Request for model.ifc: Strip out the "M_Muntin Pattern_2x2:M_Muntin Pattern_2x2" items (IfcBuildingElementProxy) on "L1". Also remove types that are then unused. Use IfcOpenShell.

First a look at what the model holds.

```python
import ifcopenshell
import ifcopenshell.util.element

model = ifcopenshell.open("model.ifc")
print(model.schema)
storey = next(s for s in model.by_type("IfcBuildingStorey") if s.Name == "L1")
proxies = [e for e in ifcopenshell.util.element.get_decomposition(storey) if e.is_a("IfcBuildingElementProxy")]
seen = {}
for e in proxies:
    element_type = ifcopenshell.util.element.get_type(e)
    name = element_type.Name if element_type not in (None, e) else None
    seen[name] = seen.get(name, 0) + 1
for name, count in sorted(seen.items(), key=str):
    print(count, "x", name)
```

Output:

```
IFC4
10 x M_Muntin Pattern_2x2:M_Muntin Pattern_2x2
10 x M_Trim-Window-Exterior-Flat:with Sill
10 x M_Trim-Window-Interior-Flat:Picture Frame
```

```python
import ifcopenshell
import ifcopenshell.api.root
import ifcopenshell.util.element

model = ifcopenshell.open("model.ifc")

storey = next(s for s in model.by_type("IfcBuildingStorey") if s.Name == "L1")
proxies = [e for e in ifcopenshell.util.element.get_decomposition(storey) if e.is_a("IfcBuildingElementProxy")]
targets = [e for e in proxies if (t := ifcopenshell.util.element.get_type(e)) not in (None, e) and t.Name == "M_Muntin Pattern_2x2:M_Muntin Pattern_2x2"]
types = {ifcopenshell.util.element.get_type(e) for e in targets} - {None, *targets}

for e in targets:
    ifcopenshell.api.root.remove_product(model, product=e)
print(len(targets), "removed")

unused = [t for t in types if not ifcopenshell.util.element.get_types(t)]
for t in unused:
    ifcopenshell.api.root.remove_product(model, product=t)
print(len(unused), "unused types removed")

model.write("model_v2.ifc")
```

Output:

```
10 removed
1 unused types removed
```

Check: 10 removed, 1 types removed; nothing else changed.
